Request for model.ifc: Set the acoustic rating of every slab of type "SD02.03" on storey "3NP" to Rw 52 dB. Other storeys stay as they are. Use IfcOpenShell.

First a look at what the model holds.

```python
import ifcopenshell
import ifcopenshell.util.element

model = ifcopenshell.open("model.ifc")
print(model.schema)
storey = next(s for s in model.by_type("IfcBuildingStorey") if s.Name == "3NP")
slabs = [e for e in ifcopenshell.util.element.get_decomposition(storey) if e.is_a("IfcSlab")]
seen = {}
for e in slabs:
    element_type = ifcopenshell.util.element.get_type(e)
    key = (element_type.Name if element_type != e and element_type else None, ifcopenshell.util.element.get_pset(e, "Pset_SlabCommon", "AcousticRating"))
    seen[key] = seen.get(key, 0) + 1
for (name, value), count in sorted(seen.items(), key=str):
    print(count, "x", name, "|", value)
```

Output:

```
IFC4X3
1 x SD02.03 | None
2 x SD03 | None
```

```python
import ifcopenshell
import ifcopenshell.api.pset
import ifcopenshell.util.element

model = ifcopenshell.open("model.ifc")

storey = next(s for s in model.by_type("IfcBuildingStorey") if s.Name == "3NP")
slabs = [e for e in ifcopenshell.util.element.get_decomposition(storey) if e.is_a("IfcSlab")]

count = 0
for e in slabs:
    element_type = ifcopenshell.util.element.get_type(e)
    if element_type in (None, e) or element_type.Name != "SD02.03":
        continue
    # add_pset returns the element's existing set when there is one.
    pset = ifcopenshell.api.pset.add_pset(model, product=e, name="Pset_SlabCommon")
    ifcopenshell.api.pset.edit_pset(model, pset=pset, properties={"AcousticRating": "Rw 52 dB"})
    count += 1

print(count, "slabs updated")

model.write("model-out.ifc")
```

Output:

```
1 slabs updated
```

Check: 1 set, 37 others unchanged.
